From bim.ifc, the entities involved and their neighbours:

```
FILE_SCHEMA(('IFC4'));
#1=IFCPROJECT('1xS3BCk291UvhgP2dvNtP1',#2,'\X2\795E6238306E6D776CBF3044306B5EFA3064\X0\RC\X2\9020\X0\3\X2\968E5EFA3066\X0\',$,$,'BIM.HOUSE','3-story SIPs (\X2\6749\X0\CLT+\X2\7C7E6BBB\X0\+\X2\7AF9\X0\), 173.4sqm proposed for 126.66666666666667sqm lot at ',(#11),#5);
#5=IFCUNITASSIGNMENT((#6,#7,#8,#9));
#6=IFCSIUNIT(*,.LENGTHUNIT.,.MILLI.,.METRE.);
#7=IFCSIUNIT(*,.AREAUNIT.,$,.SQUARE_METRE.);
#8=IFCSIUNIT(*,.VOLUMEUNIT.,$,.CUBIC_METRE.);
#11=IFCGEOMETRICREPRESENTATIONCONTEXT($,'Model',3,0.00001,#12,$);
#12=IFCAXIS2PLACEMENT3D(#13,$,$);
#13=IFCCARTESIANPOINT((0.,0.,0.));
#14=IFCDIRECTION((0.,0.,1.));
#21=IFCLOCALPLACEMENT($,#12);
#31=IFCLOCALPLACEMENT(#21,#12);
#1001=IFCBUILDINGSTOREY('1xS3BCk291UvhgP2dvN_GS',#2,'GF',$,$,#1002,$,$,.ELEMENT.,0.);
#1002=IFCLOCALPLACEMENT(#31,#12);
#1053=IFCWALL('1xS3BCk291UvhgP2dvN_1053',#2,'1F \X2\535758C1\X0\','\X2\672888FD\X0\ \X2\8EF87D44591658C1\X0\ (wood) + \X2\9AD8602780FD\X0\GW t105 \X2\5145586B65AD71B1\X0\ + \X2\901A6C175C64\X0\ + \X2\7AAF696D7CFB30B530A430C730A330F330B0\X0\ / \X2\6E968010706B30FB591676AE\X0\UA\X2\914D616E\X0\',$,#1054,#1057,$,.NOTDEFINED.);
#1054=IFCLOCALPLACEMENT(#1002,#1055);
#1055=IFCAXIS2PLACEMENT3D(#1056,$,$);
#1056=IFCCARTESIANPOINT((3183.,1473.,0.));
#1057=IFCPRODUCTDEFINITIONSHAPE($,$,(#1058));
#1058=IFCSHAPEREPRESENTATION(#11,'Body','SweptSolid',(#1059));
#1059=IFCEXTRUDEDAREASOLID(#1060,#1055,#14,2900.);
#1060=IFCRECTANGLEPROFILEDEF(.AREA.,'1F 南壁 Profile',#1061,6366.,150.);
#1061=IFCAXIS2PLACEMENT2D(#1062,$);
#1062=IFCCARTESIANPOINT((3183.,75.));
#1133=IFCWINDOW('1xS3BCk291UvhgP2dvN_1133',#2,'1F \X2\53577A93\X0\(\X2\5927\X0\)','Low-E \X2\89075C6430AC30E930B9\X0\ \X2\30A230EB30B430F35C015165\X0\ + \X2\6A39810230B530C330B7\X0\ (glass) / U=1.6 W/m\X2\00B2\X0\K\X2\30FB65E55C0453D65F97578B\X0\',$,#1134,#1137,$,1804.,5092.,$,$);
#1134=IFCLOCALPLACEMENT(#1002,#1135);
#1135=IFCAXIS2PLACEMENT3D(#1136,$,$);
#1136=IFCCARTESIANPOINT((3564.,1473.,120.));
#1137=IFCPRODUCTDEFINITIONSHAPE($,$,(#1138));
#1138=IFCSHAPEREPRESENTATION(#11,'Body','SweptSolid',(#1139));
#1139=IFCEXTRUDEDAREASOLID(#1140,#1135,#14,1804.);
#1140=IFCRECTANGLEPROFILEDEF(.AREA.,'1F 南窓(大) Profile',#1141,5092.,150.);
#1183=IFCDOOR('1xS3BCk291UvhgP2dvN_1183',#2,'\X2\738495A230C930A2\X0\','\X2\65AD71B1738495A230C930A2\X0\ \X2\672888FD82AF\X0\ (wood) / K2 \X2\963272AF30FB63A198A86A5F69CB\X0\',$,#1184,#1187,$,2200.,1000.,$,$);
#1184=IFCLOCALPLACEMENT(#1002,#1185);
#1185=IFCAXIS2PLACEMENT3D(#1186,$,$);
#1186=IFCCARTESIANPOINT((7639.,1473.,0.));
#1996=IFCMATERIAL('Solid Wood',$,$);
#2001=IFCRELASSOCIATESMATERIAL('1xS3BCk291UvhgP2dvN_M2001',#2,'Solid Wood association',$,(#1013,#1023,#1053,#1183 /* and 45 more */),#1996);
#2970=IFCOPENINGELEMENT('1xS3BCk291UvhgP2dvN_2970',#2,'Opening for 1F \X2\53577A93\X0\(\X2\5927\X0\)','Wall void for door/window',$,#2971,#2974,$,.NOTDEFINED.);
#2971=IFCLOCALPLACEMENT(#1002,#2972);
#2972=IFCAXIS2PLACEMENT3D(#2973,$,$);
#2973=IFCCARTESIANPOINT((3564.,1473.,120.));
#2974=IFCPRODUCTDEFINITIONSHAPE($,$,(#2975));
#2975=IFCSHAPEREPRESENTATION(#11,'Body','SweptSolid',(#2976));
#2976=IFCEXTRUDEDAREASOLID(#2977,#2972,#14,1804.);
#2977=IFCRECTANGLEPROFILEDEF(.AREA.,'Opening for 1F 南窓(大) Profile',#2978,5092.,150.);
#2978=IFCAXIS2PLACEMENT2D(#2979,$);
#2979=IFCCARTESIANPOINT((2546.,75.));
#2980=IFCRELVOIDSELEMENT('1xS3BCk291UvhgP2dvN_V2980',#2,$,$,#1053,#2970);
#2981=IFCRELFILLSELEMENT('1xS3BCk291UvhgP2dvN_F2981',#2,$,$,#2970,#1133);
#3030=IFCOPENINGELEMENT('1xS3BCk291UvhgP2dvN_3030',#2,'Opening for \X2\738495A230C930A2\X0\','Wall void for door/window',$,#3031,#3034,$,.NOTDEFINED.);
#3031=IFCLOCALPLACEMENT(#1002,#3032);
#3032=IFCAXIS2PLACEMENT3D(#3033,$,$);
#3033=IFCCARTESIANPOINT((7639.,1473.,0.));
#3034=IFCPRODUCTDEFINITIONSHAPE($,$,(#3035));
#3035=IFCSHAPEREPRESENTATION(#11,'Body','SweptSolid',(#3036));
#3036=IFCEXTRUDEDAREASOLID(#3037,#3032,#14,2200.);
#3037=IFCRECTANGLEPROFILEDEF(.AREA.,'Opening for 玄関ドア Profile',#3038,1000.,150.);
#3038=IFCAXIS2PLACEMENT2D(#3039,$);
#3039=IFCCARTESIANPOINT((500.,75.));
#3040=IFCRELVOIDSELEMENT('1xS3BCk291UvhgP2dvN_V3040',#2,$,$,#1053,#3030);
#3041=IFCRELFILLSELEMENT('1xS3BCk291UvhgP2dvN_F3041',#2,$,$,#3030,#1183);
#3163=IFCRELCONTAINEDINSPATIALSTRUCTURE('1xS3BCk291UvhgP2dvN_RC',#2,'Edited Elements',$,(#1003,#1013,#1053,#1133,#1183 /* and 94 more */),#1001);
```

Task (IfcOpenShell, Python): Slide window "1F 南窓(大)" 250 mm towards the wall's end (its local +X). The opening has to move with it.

```python
import ifcopenshell
import ifcopenshell.api.geometry
import ifcopenshell.util.placement
import ifcopenshell.util.unit

model = ifcopenshell.open("bim.ifc")
unit_scale = ifcopenshell.util.unit.calculate_unit_scale(model)

window = model.by_guid("1xS3BCk291UvhgP2dvN_1133")
opening = window.FillsVoids[0].RelatingOpeningElement
wall = opening.VoidsElements[0].RelatingBuildingElement

wall_matrix = ifcopenshell.util.placement.get_local_placement(wall.ObjectPlacement)
shift = wall_matrix[:3, 0] * 0.25 / unit_scale
before = ifcopenshell.util.placement.get_local_placement(window.ObjectPlacement)[:3, 3].copy()

# The window is not placed relative to its opening, so move both.
for product in (opening, window):
    matrix = ifcopenshell.util.placement.get_local_placement(product.ObjectPlacement)
    matrix[:3, 3] += shift
    ifcopenshell.api.geometry.edit_object_placement(model, product=product, matrix=matrix, is_si=False)

after = ifcopenshell.util.placement.get_local_placement(window.ObjectPlacement)[:3, 3]
print("window moved by", (after - before).round(3) + 0.0)

model.write("bim_v2.ifc")
```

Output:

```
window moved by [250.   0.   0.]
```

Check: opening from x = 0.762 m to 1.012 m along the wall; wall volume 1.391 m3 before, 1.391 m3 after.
